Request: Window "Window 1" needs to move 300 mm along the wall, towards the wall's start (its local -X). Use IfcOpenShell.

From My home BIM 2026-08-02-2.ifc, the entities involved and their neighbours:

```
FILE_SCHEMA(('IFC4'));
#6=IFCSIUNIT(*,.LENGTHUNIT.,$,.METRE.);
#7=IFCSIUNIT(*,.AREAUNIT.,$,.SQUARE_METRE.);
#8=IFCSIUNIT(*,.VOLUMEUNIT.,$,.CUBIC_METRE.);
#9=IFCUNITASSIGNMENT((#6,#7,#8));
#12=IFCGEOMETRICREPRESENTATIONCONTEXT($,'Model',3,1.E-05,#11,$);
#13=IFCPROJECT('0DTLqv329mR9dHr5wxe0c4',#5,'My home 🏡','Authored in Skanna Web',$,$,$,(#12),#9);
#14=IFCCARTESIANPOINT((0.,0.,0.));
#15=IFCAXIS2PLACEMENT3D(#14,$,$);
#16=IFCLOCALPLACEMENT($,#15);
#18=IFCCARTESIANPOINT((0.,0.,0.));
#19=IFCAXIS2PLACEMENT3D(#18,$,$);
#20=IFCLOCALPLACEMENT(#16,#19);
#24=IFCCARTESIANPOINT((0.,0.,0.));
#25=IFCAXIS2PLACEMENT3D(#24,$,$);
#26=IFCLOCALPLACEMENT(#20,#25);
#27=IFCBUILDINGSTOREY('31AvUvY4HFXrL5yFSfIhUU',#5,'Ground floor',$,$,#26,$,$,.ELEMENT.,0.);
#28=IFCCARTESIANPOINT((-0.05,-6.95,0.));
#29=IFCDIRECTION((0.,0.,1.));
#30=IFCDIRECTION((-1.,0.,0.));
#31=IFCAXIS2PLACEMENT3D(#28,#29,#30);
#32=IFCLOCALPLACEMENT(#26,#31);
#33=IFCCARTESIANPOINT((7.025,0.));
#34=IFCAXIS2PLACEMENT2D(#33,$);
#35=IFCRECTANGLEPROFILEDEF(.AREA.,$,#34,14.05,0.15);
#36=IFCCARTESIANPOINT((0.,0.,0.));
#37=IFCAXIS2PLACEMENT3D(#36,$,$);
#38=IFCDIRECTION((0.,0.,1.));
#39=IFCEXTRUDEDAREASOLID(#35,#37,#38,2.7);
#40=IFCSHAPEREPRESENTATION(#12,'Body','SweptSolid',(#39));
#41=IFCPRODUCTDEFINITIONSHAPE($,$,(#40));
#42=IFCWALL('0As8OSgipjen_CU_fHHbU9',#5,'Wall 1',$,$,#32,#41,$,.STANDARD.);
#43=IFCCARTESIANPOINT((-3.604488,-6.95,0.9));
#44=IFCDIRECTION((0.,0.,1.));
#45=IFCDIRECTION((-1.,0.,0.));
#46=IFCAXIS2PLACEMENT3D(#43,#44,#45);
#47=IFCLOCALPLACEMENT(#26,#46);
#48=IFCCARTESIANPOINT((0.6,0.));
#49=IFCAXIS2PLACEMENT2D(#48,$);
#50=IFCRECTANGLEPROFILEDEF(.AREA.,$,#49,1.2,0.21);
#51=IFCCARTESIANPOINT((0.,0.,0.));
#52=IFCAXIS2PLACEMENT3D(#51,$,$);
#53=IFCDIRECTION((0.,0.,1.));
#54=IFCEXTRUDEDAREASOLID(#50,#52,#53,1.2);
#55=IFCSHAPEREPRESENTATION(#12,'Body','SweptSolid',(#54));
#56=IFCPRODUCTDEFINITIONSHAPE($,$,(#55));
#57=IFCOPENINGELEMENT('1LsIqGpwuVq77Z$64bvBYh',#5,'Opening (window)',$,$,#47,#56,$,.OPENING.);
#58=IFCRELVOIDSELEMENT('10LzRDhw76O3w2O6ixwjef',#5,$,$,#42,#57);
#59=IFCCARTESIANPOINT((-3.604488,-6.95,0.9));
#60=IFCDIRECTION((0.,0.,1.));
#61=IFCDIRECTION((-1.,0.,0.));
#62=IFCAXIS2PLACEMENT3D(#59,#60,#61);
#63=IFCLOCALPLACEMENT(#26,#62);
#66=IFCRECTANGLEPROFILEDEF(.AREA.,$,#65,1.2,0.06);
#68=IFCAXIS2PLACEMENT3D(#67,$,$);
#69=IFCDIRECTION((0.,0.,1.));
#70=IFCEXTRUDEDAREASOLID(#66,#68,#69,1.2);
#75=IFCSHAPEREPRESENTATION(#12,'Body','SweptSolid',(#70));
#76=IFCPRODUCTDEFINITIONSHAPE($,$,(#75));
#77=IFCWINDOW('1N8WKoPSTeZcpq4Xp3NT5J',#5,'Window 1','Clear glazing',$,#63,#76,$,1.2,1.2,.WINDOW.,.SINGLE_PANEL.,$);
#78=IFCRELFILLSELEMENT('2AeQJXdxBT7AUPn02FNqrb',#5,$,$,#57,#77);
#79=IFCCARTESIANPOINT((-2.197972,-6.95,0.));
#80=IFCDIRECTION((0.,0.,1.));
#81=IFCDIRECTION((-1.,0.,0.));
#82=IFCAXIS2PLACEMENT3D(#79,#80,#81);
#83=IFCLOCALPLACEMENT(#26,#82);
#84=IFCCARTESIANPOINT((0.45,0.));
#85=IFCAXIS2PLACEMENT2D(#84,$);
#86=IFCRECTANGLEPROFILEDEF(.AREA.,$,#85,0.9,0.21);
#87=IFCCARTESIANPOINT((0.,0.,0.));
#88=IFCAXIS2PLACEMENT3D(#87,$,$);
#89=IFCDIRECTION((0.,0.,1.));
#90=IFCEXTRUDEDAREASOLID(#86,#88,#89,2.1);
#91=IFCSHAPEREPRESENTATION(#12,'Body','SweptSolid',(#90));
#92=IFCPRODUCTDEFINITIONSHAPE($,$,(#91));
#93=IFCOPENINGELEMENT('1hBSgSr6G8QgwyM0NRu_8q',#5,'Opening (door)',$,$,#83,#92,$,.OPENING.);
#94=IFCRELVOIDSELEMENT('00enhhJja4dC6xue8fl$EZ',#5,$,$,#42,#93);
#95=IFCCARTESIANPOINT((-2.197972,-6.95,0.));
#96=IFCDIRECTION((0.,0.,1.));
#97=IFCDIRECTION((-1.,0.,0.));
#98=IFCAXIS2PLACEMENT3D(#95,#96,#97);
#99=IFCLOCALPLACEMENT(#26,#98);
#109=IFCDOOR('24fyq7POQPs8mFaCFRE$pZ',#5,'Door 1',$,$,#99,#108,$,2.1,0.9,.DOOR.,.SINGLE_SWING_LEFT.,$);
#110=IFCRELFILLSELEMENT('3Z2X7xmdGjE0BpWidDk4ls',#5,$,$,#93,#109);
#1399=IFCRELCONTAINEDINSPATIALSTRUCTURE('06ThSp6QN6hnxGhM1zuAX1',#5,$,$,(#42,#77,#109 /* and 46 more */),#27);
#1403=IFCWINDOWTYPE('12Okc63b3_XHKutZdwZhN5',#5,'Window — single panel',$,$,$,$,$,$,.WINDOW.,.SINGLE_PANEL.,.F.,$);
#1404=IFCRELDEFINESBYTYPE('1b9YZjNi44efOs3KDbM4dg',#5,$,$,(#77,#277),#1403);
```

```python
import ifcopenshell
import ifcopenshell.api.geometry
import ifcopenshell.util.placement
import ifcopenshell.util.unit

model = ifcopenshell.open("My home BIM 2026-08-02-2.ifc")
unit_scale = ifcopenshell.util.unit.calculate_unit_scale(model)

window = model.by_id(77)
opening = window.FillsVoids[0].RelatingOpeningElement
wall = opening.VoidsElements[0].RelatingBuildingElement

wall_matrix = ifcopenshell.util.placement.get_local_placement(wall.ObjectPlacement)
shift = wall_matrix[:3, 0] * -0.3 / unit_scale
before = ifcopenshell.util.placement.get_local_placement(window.ObjectPlacement)[:3, 3].copy()

# The window is not placed relative to its opening, so move both.
for product in (opening, window):
    matrix = ifcopenshell.util.placement.get_local_placement(product.ObjectPlacement)
    matrix[:3, 3] += shift
    ifcopenshell.api.geometry.edit_object_placement(model, product=product, matrix=matrix, is_si=False)

after = ifcopenshell.util.placement.get_local_placement(window.ObjectPlacement)[:3, 3]
print("window moved by", (after - before).round(3) + 0.0)

model.write("My home BIM 2026-08-02-2_edited.ifc")
```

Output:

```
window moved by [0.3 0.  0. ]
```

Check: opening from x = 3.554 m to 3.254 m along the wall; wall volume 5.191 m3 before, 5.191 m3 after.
